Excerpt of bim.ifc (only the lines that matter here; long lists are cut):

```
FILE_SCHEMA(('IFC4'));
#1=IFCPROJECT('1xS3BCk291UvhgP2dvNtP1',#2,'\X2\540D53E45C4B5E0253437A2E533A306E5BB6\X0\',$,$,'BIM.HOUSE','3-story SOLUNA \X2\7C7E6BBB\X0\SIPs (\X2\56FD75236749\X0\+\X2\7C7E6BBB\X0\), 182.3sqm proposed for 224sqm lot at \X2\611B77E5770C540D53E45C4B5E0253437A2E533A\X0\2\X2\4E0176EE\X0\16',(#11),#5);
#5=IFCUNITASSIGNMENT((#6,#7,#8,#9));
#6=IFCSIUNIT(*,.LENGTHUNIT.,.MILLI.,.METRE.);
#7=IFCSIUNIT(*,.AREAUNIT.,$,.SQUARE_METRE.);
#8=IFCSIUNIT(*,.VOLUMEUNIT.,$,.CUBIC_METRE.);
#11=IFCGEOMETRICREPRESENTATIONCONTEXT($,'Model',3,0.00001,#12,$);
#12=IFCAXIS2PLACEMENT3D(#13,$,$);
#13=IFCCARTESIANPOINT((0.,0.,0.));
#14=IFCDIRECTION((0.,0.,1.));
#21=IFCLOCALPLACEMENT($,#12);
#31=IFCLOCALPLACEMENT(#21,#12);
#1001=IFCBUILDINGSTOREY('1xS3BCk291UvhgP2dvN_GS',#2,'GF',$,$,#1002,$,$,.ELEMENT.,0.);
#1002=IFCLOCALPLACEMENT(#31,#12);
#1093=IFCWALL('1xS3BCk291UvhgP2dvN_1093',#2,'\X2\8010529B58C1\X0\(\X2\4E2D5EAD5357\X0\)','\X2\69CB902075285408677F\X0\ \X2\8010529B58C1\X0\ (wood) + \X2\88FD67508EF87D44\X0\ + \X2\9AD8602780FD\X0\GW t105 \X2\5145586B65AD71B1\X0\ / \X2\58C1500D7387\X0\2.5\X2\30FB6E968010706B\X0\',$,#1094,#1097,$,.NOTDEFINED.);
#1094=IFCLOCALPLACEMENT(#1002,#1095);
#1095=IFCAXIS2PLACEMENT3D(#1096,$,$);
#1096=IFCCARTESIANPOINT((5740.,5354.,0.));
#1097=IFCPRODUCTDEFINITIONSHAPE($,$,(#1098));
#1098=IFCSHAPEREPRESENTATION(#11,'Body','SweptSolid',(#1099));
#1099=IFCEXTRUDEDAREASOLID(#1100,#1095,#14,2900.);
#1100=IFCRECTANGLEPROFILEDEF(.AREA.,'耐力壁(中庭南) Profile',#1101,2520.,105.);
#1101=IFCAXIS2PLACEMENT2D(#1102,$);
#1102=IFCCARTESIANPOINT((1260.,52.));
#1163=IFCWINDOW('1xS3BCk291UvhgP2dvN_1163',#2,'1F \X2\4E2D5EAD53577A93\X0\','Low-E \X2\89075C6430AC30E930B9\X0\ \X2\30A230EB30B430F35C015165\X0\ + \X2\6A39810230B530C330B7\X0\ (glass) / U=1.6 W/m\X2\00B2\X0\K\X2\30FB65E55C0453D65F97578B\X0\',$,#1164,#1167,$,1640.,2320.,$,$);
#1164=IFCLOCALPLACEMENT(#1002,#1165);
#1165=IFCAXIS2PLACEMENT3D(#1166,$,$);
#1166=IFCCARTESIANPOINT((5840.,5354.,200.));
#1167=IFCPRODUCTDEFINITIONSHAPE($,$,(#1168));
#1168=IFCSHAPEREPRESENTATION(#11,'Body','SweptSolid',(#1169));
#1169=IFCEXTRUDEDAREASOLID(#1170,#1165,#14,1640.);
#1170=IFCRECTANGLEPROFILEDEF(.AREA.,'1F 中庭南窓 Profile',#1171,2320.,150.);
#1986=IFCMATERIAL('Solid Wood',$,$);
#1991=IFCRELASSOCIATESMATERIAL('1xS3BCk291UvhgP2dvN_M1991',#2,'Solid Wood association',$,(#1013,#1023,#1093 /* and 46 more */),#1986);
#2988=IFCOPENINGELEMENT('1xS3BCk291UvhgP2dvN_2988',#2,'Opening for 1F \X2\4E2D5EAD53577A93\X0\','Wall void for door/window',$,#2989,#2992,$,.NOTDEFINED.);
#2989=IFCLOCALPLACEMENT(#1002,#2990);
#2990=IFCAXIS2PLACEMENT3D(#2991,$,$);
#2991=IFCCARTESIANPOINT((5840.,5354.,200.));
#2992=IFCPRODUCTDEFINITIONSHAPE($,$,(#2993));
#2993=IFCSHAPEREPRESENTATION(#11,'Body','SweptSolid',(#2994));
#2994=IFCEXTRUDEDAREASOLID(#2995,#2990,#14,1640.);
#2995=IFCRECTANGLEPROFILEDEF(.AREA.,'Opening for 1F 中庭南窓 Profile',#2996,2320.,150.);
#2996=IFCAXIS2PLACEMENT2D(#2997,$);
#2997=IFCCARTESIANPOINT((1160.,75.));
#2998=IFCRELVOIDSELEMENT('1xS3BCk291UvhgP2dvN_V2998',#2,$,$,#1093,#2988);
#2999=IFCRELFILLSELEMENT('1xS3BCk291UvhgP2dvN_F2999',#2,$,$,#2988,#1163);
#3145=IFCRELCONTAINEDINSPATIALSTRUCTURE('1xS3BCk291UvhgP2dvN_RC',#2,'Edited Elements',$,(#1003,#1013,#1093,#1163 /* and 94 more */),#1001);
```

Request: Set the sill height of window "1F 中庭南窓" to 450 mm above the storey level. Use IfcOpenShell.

```python
import numpy as np
import ifcopenshell
import ifcopenshell.api.geometry
import ifcopenshell.geom
import ifcopenshell.util.element
import ifcopenshell.util.placement
import ifcopenshell.util.shape
import ifcopenshell.util.unit

model = ifcopenshell.open("bim.ifc")
unit_scale = ifcopenshell.util.unit.calculate_unit_scale(model)

window = model.by_guid("1xS3BCk291UvhgP2dvN_1163")
opening = window.FillsVoids[0].RelatingOpeningElement
storey = ifcopenshell.util.element.get_container(window, ifc_class="IfcBuildingStorey")
level = ifcopenshell.util.placement.get_local_placement(storey.ObjectPlacement)[2, 3]

# The opening's origin need not be at the sill, so measure its lowest point.
shape = ifcopenshell.geom.create_shape(ifcopenshell.geom.settings(), opening)
bottom = ifcopenshell.util.shape.get_shape_bottom_elevation(shape, shape.geometry) / unit_scale
dz = level + 0.45 / unit_scale - bottom

shift = np.array([0.0, 0.0, dz])
# The window is not placed relative to its opening, so move both.
for product in (opening, window):
    matrix = ifcopenshell.util.placement.get_local_placement(product.ObjectPlacement)
    matrix[:3, 3] += shift
    ifcopenshell.api.geometry.edit_object_placement(model, product=product, matrix=matrix, is_si=False)

print(f"moved by {dz * unit_scale:+.3f} m")

model.write("bim-out.ifc")
```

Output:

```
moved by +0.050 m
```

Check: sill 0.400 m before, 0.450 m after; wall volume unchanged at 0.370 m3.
